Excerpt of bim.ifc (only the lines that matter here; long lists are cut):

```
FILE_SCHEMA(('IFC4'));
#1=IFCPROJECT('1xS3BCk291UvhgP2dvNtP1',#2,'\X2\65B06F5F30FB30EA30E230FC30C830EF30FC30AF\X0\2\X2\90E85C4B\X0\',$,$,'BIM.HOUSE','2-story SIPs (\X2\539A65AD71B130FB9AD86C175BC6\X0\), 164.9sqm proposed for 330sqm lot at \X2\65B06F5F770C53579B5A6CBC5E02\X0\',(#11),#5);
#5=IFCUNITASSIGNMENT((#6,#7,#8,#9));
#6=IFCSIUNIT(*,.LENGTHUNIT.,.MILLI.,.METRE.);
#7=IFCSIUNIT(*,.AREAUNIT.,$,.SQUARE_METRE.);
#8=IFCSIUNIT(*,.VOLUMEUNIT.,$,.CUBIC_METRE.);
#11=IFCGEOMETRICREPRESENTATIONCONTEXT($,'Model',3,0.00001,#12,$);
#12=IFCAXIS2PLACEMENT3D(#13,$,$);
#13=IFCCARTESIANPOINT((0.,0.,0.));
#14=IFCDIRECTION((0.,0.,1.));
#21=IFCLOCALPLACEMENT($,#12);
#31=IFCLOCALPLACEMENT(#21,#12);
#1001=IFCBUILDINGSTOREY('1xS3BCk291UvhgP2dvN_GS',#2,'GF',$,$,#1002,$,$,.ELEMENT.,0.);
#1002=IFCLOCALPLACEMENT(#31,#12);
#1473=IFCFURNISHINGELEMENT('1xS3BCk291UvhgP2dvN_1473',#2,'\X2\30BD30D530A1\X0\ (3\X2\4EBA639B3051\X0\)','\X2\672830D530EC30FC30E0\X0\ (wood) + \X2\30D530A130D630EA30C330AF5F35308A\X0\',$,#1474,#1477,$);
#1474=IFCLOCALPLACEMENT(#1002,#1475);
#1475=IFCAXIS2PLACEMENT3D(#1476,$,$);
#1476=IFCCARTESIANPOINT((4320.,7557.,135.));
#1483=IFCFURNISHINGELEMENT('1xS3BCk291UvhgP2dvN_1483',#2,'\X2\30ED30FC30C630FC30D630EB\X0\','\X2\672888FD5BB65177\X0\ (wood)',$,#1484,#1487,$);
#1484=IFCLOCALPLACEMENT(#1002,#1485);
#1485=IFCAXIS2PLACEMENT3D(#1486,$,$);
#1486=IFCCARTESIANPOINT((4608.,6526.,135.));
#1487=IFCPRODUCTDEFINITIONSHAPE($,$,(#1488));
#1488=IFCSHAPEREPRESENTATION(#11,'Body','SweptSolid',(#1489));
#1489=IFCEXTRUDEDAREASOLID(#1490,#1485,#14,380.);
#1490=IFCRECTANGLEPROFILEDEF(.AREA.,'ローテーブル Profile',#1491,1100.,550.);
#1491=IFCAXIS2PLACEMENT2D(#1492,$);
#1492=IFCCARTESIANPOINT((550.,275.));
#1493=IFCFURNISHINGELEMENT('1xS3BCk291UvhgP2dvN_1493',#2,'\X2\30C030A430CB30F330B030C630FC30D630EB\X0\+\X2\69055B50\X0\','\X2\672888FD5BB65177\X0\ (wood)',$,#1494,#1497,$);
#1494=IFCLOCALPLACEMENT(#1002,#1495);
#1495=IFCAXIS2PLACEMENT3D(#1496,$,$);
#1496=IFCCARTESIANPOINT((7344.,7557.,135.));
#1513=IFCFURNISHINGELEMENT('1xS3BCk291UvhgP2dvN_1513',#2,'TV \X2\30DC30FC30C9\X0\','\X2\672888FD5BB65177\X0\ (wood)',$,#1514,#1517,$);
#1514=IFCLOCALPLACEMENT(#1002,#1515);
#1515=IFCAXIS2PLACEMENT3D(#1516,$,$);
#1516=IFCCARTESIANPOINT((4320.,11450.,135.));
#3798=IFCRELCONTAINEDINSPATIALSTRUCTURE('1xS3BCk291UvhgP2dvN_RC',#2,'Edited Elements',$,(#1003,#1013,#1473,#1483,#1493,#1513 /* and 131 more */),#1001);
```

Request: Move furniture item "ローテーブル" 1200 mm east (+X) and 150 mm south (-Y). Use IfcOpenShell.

```python
import ifcopenshell
import ifcopenshell.api.geometry
import ifcopenshell.util.placement

model = ifcopenshell.open("bim.ifc")

item = model.by_guid("1xS3BCk291UvhgP2dvN_1483")
matrix = ifcopenshell.util.placement.get_local_placement(item.ObjectPlacement)
matrix[0, 3] += 1200.0
matrix[1, 3] -= 150.0
ifcopenshell.api.geometry.edit_object_placement(model, product=item, matrix=matrix, is_si=False)

print(ifcopenshell.util.placement.get_local_placement(item.ObjectPlacement).round(3) + 0.0)

model.write("bim-out.ifc")
```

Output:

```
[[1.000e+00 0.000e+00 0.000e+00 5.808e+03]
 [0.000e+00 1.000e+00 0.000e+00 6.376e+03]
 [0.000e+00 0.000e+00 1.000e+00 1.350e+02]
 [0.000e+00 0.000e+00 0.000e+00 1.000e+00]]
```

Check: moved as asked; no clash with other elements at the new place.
